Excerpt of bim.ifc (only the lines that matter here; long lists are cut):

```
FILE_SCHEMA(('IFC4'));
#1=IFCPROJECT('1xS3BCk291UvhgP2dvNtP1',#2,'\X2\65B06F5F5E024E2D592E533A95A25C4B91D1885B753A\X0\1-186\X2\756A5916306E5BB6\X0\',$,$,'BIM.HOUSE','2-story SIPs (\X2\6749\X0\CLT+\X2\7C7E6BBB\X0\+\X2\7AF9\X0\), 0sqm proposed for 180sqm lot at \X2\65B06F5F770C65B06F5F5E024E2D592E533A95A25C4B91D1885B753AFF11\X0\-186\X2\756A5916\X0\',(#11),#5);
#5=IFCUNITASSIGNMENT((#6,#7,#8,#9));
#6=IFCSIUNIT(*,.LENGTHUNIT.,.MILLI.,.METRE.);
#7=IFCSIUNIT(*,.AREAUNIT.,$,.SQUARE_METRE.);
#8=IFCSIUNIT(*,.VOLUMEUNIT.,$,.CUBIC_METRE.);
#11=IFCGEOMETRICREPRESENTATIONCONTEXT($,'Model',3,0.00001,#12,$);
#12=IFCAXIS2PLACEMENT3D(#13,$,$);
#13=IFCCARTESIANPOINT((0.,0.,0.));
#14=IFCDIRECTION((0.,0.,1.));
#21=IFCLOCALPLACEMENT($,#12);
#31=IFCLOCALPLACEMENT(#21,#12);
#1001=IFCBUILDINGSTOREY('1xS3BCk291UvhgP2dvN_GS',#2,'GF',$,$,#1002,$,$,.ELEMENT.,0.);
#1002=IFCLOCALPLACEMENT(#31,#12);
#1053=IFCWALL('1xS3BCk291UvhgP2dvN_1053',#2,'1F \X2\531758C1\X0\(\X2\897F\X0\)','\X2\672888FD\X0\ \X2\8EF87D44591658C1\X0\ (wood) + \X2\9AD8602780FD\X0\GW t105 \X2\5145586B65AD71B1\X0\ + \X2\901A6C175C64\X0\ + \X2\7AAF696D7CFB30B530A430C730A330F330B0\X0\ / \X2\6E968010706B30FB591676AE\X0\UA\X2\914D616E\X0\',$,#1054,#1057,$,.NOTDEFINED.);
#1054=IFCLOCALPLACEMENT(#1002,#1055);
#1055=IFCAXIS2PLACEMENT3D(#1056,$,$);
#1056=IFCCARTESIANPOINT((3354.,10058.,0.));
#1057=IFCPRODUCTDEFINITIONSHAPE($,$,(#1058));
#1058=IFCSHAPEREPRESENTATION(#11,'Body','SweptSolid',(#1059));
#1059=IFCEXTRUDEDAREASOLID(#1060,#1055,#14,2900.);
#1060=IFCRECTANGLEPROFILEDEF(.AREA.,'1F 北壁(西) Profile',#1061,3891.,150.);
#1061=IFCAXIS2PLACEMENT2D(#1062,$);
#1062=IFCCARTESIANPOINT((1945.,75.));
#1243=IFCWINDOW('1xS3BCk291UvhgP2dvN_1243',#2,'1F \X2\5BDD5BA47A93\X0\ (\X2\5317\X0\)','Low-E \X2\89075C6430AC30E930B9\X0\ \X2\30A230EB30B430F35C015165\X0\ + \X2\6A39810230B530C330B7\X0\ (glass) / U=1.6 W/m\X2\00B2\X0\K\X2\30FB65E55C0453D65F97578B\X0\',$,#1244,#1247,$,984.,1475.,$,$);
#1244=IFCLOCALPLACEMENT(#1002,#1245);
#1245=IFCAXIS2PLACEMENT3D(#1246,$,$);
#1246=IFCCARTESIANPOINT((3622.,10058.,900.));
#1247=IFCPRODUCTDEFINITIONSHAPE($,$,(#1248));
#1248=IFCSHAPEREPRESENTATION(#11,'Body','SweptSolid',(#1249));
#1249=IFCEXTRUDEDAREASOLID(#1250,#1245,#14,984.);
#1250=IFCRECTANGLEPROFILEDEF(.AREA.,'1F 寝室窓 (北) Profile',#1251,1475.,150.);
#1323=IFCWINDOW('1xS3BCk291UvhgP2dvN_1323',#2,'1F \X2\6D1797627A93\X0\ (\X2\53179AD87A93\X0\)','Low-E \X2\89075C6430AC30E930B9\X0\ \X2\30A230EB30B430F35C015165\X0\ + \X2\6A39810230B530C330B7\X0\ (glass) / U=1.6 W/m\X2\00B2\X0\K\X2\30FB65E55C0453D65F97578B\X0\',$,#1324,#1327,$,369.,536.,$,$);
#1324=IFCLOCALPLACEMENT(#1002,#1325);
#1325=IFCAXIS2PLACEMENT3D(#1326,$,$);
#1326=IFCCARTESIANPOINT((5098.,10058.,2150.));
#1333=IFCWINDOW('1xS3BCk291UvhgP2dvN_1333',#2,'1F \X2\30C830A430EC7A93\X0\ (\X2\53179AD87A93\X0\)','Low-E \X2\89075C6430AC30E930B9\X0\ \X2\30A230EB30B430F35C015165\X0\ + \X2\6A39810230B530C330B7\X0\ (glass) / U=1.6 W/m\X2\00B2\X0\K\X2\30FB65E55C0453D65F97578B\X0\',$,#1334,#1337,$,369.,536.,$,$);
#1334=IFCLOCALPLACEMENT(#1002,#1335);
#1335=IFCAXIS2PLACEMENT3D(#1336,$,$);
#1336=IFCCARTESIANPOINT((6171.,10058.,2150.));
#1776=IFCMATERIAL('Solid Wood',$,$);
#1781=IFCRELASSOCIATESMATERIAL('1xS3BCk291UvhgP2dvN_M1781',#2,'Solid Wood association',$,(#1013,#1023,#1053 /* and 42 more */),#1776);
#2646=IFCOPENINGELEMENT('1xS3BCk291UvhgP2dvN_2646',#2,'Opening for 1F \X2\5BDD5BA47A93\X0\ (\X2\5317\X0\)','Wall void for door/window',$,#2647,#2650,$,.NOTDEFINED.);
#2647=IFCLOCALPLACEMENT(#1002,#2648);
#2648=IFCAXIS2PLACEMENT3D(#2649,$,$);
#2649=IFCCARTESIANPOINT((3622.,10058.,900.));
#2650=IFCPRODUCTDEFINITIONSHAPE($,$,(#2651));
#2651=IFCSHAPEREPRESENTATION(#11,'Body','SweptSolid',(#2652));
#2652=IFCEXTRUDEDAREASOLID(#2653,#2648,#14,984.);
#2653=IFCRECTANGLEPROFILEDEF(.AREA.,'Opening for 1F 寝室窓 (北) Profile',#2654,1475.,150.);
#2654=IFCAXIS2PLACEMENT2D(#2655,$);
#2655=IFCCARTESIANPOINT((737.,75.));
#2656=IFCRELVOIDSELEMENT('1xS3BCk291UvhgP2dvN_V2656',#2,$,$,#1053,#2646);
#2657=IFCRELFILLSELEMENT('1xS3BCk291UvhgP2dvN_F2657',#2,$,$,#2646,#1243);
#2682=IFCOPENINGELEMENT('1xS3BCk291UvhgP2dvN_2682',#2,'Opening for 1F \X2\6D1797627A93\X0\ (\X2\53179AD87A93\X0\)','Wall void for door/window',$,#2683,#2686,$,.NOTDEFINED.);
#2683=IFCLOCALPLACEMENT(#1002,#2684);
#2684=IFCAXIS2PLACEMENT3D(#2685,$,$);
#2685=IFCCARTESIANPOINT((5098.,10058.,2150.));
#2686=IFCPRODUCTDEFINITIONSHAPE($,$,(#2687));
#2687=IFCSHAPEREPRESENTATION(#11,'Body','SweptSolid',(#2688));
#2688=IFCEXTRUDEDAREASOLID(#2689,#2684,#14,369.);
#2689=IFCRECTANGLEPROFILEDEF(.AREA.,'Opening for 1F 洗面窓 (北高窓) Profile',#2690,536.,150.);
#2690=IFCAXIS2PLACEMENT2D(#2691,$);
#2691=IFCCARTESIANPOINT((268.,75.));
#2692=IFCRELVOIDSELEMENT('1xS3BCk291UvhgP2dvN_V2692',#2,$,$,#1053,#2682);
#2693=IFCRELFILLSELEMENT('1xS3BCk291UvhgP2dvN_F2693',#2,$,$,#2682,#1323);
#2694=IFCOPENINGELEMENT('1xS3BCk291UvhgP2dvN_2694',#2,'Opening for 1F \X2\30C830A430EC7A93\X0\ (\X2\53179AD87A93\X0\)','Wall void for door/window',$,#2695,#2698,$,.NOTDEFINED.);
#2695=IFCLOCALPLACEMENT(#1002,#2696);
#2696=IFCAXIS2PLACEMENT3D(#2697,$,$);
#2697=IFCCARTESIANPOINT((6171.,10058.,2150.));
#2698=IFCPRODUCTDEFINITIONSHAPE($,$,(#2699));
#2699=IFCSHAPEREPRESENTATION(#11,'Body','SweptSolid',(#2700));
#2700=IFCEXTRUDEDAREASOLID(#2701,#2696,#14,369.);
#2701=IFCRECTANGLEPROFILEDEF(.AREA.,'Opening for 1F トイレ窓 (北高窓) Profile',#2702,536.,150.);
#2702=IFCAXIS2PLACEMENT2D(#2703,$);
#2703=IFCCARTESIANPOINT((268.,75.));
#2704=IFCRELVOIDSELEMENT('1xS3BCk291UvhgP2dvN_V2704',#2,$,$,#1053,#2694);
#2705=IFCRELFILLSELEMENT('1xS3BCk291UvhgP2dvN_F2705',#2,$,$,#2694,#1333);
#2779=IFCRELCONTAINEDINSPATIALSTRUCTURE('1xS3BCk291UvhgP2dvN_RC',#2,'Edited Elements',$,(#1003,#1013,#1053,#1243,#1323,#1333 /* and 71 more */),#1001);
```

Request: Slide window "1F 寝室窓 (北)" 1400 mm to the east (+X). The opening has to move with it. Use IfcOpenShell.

```python
import ifcopenshell
import ifcopenshell.api.geometry
import ifcopenshell.util.placement
import ifcopenshell.util.unit

model = ifcopenshell.open("bim.ifc")
unit_scale = ifcopenshell.util.unit.calculate_unit_scale(model)

window = model.by_guid("1xS3BCk291UvhgP2dvN_1243")
opening = window.FillsVoids[0].RelatingOpeningElement
wall = opening.VoidsElements[0].RelatingBuildingElement

wall_matrix = ifcopenshell.util.placement.get_local_placement(wall.ObjectPlacement)
shift = wall_matrix[:3, 0] * 1.4 / unit_scale
before = ifcopenshell.util.placement.get_local_placement(window.ObjectPlacement)[:3, 3].copy()

# The window is not placed relative to its opening, so move both.
for product in (opening, window):
    matrix = ifcopenshell.util.placement.get_local_placement(product.ObjectPlacement)
    matrix[:3, 3] += shift
    ifcopenshell.api.geometry.edit_object_placement(model, product=product, matrix=matrix, is_si=False)

after = ifcopenshell.util.placement.get_local_placement(window.ObjectPlacement)[:3, 3]
print("window moved by", (after - before).round(3) + 0.0)

model.write("bim_updated.ifc")
```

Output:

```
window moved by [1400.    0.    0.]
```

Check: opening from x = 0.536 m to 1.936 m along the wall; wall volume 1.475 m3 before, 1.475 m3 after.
